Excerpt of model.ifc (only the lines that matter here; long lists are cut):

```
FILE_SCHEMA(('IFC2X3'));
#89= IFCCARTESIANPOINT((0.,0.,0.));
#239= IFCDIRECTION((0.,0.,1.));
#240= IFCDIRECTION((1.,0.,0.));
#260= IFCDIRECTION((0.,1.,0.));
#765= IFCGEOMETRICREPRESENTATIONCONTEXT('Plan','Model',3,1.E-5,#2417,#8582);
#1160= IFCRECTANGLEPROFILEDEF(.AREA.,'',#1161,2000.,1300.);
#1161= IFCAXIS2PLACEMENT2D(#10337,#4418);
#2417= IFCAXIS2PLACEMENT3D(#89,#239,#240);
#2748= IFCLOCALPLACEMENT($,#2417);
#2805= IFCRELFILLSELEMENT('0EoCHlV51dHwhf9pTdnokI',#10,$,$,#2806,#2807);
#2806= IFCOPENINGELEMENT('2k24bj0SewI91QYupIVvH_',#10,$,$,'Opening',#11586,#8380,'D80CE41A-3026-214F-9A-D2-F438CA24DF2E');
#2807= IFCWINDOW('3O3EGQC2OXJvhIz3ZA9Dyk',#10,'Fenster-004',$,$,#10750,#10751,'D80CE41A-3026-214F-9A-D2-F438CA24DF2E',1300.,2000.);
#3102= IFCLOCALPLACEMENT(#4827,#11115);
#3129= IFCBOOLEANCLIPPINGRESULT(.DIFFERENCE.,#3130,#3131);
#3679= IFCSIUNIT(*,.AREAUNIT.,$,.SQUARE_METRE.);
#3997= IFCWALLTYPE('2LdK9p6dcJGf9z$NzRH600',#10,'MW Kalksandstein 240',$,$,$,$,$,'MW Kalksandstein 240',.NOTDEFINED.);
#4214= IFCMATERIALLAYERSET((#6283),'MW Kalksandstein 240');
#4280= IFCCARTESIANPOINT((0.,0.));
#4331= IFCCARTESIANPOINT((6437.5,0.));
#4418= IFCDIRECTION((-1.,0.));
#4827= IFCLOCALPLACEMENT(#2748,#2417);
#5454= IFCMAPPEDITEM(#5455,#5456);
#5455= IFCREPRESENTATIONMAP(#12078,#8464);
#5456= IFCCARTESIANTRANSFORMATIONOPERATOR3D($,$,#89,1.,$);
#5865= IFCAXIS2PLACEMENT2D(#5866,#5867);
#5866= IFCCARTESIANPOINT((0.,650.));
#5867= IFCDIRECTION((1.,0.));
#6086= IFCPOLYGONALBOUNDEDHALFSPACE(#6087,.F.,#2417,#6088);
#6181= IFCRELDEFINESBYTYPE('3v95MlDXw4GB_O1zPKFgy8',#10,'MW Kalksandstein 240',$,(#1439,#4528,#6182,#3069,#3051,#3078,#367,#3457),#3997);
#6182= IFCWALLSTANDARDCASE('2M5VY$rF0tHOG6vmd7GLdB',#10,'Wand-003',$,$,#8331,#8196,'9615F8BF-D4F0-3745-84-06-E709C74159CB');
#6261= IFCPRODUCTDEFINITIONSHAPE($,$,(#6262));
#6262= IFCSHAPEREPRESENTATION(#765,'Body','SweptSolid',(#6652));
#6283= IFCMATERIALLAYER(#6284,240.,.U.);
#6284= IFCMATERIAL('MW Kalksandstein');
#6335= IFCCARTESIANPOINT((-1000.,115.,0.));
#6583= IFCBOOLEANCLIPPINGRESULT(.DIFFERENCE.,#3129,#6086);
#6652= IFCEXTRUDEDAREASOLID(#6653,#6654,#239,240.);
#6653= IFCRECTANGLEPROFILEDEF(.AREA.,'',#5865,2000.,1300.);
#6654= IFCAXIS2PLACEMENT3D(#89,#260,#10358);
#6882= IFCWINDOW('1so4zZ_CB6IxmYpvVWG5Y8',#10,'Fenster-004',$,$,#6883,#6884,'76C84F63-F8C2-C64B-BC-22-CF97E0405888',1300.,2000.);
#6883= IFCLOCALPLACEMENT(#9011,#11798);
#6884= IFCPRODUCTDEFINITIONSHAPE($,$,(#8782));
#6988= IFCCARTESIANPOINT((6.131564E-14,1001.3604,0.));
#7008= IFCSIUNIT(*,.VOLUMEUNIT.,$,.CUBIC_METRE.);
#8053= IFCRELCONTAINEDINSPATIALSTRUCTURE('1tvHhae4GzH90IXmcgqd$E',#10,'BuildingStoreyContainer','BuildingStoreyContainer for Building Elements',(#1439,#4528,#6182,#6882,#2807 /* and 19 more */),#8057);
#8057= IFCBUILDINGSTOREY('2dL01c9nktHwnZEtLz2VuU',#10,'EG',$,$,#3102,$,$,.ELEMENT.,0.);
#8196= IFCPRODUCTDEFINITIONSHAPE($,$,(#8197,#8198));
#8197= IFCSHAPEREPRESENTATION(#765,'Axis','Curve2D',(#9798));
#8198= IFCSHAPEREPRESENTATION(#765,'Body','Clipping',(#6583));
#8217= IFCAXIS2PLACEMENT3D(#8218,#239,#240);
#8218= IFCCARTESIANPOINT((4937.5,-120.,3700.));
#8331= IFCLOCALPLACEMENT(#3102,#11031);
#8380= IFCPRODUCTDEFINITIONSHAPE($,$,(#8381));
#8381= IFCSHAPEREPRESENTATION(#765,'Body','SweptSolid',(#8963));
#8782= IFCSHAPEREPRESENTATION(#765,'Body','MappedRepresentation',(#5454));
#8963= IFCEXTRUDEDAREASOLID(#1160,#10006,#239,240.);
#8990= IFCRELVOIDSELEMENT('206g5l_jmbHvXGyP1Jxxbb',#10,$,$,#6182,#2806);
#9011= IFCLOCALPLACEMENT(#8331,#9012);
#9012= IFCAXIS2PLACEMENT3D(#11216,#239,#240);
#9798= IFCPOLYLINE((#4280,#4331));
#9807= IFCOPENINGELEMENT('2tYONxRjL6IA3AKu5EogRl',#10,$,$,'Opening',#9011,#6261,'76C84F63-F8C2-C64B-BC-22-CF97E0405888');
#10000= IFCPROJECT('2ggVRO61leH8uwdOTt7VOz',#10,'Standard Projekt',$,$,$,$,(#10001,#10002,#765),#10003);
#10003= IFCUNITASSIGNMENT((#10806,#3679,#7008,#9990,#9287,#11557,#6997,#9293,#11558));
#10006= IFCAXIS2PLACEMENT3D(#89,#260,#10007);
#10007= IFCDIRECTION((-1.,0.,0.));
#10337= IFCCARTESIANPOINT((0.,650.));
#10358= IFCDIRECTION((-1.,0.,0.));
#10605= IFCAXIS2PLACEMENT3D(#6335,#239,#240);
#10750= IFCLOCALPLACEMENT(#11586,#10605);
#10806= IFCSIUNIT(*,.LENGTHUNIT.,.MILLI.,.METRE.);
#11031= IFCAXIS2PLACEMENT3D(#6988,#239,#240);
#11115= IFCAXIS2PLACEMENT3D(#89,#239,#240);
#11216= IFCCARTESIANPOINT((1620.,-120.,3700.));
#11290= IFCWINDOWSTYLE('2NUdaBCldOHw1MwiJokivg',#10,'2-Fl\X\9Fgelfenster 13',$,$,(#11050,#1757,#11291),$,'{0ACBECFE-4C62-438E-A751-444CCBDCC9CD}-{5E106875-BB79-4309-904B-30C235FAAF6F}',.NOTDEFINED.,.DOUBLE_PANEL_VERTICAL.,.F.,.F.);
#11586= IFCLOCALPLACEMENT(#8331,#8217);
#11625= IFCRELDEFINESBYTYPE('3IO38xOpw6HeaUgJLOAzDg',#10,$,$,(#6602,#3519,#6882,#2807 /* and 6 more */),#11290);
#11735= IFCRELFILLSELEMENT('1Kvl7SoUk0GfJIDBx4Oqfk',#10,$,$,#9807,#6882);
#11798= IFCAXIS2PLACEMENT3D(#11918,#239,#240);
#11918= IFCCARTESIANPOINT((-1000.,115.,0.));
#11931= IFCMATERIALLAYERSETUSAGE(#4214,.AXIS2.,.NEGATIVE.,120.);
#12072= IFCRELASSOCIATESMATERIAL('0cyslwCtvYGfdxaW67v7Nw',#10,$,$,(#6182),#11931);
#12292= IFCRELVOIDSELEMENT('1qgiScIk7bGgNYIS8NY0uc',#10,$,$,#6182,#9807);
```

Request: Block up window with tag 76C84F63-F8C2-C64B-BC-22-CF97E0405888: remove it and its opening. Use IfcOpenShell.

```python
import ifcopenshell
import ifcopenshell.api.feature
import ifcopenshell.api.root
import ifcopenshell.geom
import ifcopenshell.util.shape

model = ifcopenshell.open("model.ifc")
settings = ifcopenshell.geom.settings()


def volume(element):
    """Net volume in cubic metres, openings subtracted."""
    shape = ifcopenshell.geom.create_shape(settings, element)
    return ifcopenshell.util.shape.get_volume(shape.geometry)


window = model.by_guid("1so4zZ_CB6IxmYpvVWG5Y8")
opening = window.FillsVoids[0].RelatingOpeningElement
wall = opening.VoidsElements[0].RelatingBuildingElement
before = volume(wall)

ifcopenshell.api.root.remove_product(model, product=window)
ifcopenshell.api.feature.remove_feature(model, feature=opening)

after = volume(wall)

print(f"wall volume {before:.3f} -> {after:.3f} m3")

model.write("model_rev.ifc")
```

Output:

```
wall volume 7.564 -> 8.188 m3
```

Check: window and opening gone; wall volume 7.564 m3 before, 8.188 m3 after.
